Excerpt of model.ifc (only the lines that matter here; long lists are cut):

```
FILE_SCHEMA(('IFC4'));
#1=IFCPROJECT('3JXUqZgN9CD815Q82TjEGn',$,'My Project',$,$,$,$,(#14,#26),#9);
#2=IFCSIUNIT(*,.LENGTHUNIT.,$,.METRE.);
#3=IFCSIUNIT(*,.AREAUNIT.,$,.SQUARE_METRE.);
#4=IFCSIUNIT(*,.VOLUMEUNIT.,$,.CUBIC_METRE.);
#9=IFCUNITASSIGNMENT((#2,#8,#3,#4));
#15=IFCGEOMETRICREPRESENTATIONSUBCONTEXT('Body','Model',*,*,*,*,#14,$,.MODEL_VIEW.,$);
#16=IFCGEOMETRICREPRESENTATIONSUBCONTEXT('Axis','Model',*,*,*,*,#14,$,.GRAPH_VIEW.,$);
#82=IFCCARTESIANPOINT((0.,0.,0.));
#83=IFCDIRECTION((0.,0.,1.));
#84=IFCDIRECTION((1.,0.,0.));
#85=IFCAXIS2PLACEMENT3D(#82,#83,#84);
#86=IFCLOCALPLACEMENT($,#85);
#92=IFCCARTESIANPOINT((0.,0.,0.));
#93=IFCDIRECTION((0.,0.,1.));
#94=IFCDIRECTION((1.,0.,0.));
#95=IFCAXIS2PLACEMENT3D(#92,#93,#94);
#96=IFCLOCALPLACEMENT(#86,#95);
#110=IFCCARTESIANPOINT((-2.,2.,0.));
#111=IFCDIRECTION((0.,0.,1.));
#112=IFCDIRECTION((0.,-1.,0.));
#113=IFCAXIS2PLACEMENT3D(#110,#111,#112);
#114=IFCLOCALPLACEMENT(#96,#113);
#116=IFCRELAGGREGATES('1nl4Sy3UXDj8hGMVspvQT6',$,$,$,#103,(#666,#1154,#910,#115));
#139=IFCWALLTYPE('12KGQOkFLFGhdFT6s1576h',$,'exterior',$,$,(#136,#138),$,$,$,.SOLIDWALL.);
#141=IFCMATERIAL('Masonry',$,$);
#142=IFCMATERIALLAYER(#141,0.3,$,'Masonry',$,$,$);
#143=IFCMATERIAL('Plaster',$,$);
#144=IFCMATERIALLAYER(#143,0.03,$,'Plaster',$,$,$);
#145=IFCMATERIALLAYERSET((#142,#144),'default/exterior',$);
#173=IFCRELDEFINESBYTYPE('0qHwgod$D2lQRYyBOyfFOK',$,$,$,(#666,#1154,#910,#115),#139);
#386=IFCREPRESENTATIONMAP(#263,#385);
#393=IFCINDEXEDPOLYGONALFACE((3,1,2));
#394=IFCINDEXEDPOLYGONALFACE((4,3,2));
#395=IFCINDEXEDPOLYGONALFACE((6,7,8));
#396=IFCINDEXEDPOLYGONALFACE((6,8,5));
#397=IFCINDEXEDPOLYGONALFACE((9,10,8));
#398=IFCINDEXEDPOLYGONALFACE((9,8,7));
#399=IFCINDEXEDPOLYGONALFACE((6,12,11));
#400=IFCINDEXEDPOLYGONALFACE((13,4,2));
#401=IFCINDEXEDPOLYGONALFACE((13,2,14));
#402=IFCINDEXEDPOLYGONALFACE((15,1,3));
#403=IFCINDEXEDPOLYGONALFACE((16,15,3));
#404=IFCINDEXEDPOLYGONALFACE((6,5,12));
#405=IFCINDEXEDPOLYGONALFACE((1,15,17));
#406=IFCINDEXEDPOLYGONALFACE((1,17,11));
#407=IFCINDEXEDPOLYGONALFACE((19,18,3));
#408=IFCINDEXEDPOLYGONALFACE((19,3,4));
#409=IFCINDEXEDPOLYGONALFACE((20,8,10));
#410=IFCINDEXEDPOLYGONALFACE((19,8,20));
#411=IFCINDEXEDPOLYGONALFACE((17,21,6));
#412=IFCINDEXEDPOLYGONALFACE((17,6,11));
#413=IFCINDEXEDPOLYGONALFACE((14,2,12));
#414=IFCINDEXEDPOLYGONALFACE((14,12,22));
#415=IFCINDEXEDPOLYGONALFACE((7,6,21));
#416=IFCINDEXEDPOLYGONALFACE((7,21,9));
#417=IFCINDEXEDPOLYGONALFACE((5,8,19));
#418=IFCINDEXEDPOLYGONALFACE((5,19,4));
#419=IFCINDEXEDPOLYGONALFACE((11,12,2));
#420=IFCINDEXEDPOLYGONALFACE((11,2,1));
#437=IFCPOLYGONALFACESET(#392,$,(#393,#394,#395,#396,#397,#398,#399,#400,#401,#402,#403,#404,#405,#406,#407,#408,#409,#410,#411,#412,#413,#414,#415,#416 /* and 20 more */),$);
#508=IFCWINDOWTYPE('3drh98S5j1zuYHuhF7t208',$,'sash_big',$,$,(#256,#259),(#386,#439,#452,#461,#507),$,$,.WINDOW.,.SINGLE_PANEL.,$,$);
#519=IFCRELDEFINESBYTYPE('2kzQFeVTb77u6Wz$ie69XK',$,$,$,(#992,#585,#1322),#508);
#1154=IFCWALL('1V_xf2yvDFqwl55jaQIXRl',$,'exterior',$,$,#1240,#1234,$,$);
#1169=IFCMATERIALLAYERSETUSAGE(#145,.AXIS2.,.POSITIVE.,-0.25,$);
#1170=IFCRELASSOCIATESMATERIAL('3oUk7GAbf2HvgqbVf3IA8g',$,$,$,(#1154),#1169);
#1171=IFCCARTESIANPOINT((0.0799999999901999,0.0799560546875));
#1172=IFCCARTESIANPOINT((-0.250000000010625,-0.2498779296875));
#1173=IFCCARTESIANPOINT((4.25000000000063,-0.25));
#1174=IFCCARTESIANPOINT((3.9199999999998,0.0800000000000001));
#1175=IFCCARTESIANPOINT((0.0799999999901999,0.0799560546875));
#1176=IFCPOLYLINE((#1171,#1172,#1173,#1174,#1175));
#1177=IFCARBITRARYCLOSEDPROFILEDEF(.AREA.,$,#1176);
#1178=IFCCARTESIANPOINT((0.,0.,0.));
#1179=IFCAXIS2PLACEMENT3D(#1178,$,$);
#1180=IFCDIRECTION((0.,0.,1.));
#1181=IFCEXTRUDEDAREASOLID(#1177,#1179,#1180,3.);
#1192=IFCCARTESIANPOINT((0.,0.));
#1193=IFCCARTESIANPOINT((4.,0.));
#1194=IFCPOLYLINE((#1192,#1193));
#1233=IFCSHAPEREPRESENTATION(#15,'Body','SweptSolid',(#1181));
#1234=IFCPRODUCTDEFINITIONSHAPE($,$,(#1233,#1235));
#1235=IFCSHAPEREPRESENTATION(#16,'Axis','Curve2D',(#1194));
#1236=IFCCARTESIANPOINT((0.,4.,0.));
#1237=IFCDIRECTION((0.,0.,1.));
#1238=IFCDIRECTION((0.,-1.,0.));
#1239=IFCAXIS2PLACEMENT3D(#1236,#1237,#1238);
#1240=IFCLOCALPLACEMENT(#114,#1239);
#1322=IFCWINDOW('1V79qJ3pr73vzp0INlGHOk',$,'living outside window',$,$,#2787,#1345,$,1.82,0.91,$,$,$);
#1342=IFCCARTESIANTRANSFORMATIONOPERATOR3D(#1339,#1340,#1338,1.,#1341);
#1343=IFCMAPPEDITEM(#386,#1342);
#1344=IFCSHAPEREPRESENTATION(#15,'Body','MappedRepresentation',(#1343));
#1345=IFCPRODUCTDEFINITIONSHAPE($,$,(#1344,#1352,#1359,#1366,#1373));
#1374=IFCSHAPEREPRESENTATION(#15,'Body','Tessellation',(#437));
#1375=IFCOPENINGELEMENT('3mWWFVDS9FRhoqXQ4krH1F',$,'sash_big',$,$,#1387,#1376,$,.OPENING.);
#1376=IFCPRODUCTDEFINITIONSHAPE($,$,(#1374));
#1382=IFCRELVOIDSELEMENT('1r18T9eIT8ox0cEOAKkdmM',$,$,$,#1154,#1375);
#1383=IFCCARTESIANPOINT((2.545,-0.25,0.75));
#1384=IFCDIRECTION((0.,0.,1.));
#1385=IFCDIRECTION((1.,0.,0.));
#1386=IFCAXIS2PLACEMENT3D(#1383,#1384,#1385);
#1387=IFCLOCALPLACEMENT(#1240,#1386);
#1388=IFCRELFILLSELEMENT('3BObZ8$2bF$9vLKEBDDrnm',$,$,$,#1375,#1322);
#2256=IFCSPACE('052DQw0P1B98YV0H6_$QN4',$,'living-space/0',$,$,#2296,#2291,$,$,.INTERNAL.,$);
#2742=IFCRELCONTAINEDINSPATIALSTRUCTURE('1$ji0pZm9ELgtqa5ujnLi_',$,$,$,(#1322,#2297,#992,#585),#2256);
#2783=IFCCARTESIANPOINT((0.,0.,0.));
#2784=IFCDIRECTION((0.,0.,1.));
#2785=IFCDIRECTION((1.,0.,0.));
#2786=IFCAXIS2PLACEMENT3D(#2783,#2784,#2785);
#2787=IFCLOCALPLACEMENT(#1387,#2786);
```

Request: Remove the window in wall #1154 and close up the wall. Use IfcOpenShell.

```python
import ifcopenshell
import ifcopenshell.api.feature
import ifcopenshell.api.root
import ifcopenshell.geom
import ifcopenshell.util.shape

model = ifcopenshell.open("model.ifc")
settings = ifcopenshell.geom.settings()


def volume(element):
    """Net volume in cubic metres, openings subtracted."""
    shape = ifcopenshell.geom.create_shape(settings, element)
    return ifcopenshell.util.shape.get_volume(shape.geometry)


window = model.by_guid("1V79qJ3pr73vzp0INlGHOk")
opening = window.FillsVoids[0].RelatingOpeningElement
wall = opening.VoidsElements[0].RelatingBuildingElement
before = volume(wall)

ifcopenshell.api.root.remove_product(model, product=window)
ifcopenshell.api.feature.remove_feature(model, feature=opening)

after = volume(wall)

print(f"wall volume {before:.3f} -> {after:.3f} m3")

model.write("model-out.ifc")
```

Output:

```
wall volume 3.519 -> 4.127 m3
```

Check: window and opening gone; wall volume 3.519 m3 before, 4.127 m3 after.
